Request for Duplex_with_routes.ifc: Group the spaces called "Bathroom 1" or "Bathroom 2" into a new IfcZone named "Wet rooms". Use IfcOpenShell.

First a look at what the model holds.

```python
import ifcopenshell

model = ifcopenshell.open("Duplex_with_routes.ifc")
print(model.schema)
seen = {}
for space in model.by_type("IfcSpace"):
    seen[space.LongName] = seen.get(space.LongName, 0) + 1
for name, count in sorted(seen.items(), key=str):
    print(count, "x", name)
print("zones:", [z.Name for z in model.by_type("IfcZone")][:20])
```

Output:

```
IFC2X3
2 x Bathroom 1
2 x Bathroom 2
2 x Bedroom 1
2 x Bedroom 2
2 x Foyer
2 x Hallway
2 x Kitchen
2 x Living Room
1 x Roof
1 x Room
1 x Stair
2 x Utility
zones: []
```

```python
import ifcopenshell
import ifcopenshell.api.group
import ifcopenshell.api.root

model = ifcopenshell.open("Duplex_with_routes.ifc")

names = {"Bathroom 1", "Bathroom 2"}
spaces = [s for s in model.by_type("IfcSpace") if s.LongName in names]

zone = ifcopenshell.api.root.create_entity(model, ifc_class="IfcZone", name="Wet rooms")
ifcopenshell.api.group.assign_group(model, products=spaces, group=zone)
print(len(spaces), "spaces in", zone.Name)

model.write("Duplex_with_routes_rev.ifc")
```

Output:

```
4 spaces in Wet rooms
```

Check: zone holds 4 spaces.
